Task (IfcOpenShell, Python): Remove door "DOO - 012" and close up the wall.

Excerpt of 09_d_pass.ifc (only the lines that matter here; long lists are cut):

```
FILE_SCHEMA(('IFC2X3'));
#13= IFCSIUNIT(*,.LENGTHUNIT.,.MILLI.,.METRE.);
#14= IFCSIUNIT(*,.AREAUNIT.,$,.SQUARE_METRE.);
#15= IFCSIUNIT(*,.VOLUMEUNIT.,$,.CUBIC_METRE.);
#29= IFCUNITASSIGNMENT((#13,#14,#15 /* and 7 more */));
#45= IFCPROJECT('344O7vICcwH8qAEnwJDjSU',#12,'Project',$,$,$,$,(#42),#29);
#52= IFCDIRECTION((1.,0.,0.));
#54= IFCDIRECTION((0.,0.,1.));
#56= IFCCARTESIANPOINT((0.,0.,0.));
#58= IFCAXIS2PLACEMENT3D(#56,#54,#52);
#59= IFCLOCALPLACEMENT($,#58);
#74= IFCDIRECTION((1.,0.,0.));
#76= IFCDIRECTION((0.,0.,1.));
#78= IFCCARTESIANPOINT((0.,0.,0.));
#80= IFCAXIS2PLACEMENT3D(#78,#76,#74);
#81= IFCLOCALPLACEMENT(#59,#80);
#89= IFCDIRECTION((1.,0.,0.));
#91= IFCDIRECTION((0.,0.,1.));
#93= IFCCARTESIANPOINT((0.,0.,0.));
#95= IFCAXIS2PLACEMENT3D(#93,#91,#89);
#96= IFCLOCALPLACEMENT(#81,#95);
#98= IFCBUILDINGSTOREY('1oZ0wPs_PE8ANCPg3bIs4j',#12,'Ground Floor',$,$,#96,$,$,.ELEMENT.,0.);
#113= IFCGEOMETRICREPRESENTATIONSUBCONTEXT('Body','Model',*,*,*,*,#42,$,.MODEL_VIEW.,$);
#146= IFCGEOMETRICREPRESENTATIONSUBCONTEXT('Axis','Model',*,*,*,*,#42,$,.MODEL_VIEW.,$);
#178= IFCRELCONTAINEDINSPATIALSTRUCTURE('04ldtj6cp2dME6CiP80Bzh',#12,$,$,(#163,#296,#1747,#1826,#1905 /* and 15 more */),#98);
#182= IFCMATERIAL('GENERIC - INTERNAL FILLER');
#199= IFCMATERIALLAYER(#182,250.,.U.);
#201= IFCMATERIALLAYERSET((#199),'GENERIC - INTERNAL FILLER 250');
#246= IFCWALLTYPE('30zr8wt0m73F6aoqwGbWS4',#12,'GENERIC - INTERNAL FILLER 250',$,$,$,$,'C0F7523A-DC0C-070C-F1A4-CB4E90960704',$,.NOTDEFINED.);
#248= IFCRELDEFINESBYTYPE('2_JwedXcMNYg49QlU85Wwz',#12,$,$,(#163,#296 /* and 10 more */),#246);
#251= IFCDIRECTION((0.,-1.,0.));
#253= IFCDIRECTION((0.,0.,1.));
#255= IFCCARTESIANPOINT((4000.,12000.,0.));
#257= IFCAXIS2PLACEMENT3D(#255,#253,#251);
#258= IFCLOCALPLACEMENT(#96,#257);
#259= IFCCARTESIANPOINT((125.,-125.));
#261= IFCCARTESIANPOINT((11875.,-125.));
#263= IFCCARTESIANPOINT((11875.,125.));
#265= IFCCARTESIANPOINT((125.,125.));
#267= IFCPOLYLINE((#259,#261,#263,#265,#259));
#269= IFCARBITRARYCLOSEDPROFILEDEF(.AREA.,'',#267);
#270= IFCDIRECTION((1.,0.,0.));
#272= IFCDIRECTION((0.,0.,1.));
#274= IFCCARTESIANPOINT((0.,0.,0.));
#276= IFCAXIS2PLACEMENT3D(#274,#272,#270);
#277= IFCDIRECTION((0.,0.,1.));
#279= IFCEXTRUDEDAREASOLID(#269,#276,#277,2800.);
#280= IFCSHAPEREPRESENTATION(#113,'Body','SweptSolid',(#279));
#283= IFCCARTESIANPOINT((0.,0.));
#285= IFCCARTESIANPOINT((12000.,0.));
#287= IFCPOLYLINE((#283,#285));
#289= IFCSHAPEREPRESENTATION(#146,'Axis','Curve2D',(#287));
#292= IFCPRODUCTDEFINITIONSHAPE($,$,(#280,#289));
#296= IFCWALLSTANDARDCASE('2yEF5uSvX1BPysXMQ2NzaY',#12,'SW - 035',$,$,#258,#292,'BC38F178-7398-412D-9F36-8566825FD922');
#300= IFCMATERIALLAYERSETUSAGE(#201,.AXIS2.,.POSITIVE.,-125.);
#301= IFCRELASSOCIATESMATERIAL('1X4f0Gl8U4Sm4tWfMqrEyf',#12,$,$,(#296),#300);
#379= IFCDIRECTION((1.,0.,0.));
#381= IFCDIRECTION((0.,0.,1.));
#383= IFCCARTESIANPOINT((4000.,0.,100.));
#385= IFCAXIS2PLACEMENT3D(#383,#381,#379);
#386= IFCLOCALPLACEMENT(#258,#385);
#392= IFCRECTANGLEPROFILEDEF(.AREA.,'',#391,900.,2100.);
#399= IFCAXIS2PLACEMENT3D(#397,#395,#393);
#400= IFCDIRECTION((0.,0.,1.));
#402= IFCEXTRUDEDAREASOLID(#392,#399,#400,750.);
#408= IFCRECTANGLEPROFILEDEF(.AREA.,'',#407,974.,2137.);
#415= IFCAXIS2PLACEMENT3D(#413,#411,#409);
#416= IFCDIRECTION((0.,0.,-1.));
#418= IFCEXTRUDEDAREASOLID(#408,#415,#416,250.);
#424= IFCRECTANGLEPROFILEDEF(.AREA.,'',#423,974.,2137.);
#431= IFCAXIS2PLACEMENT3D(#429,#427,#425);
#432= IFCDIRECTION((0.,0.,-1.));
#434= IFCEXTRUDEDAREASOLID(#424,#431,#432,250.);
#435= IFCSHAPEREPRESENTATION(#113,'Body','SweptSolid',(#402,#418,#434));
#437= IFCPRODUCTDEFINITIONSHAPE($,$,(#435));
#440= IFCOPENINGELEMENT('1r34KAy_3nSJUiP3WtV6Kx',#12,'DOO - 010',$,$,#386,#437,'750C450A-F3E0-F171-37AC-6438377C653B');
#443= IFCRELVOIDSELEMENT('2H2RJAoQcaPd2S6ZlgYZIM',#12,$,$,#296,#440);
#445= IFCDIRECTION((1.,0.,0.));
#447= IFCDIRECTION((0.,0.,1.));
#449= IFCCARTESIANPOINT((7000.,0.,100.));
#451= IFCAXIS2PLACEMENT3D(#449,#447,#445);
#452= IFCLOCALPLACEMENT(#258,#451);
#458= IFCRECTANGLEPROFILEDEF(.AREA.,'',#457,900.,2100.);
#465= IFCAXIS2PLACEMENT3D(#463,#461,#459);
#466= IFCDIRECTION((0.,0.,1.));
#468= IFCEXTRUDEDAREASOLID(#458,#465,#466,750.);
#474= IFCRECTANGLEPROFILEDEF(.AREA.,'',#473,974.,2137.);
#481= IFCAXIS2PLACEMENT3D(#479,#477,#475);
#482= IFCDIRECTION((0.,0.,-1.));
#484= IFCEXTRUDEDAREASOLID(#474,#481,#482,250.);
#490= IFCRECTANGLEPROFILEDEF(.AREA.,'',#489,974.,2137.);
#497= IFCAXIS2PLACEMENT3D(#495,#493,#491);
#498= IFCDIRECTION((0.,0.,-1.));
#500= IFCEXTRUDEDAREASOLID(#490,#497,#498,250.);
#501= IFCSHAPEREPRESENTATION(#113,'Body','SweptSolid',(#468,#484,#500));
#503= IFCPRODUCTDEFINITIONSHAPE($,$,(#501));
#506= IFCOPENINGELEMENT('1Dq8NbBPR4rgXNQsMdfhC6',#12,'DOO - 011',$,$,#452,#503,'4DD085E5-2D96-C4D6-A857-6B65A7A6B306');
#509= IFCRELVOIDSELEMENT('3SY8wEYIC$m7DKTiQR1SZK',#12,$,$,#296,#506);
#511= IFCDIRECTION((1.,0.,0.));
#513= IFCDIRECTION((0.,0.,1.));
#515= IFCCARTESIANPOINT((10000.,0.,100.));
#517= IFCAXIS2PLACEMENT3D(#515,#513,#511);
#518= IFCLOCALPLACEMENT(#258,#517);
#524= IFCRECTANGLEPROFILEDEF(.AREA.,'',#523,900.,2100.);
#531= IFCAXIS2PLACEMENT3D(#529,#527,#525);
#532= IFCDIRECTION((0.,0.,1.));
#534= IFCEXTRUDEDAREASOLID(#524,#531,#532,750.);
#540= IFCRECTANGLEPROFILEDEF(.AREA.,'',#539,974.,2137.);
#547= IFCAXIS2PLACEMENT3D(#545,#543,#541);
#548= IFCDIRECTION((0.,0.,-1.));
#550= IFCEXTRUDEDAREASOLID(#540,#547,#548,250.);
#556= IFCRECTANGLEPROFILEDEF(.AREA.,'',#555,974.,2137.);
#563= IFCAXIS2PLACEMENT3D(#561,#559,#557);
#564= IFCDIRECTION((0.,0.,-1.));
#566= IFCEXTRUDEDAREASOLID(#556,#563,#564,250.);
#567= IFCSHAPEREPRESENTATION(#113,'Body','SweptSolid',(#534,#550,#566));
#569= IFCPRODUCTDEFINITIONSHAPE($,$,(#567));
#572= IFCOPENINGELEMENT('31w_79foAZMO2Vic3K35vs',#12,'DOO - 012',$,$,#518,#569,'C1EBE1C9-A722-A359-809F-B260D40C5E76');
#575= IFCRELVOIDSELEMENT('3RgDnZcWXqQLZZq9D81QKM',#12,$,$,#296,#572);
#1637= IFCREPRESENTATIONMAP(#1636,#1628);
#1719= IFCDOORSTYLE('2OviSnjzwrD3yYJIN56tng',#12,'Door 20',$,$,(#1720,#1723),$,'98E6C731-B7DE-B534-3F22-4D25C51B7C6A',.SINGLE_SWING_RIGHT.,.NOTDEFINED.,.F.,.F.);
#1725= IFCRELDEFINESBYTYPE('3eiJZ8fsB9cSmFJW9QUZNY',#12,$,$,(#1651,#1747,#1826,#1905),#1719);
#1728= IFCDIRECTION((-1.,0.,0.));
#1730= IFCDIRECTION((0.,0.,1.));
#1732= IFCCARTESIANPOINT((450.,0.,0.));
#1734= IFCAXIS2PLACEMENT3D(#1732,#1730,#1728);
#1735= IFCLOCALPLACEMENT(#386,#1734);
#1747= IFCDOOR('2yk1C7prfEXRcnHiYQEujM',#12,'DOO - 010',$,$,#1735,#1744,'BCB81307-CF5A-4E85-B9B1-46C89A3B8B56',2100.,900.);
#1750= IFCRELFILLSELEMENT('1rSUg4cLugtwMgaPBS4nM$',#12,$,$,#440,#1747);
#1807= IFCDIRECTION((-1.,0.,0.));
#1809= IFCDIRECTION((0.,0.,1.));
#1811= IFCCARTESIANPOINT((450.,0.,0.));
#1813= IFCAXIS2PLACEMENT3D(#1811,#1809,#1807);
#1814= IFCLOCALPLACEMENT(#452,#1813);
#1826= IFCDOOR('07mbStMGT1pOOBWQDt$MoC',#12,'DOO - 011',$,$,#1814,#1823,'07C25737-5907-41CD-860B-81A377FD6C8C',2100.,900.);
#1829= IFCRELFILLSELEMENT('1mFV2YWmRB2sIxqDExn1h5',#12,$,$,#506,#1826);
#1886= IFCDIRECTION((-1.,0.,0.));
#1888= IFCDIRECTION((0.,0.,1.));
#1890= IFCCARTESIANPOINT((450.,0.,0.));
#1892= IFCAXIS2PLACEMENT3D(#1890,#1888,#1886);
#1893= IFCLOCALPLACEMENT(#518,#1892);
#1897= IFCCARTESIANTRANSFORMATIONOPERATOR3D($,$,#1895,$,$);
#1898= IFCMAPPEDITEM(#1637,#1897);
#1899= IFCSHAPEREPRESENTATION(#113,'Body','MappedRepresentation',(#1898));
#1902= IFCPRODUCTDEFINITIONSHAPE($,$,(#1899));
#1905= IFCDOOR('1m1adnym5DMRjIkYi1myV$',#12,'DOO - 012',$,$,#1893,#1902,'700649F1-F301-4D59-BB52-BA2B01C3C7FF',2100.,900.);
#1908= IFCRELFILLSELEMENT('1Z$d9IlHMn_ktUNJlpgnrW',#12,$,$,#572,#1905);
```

```python
import ifcopenshell
import ifcopenshell.api.feature
import ifcopenshell.api.root
import ifcopenshell.geom
import ifcopenshell.util.shape

model = ifcopenshell.open("09_d_pass.ifc")
settings = ifcopenshell.geom.settings()


def volume(element):
    """Net volume in cubic metres, openings subtracted."""
    shape = ifcopenshell.geom.create_shape(settings, element)
    return ifcopenshell.util.shape.get_volume(shape.geometry)


door = model.by_guid("1m1adnym5DMRjIkYi1myV$")
opening = door.FillsVoids[0].RelatingOpeningElement
wall = opening.VoidsElements[0].RelatingBuildingElement
before = volume(wall)

ifcopenshell.api.root.remove_product(model, product=door)
ifcopenshell.api.feature.remove_feature(model, feature=opening)

after = volume(wall)

print(f"wall volume {before:.3f} -> {after:.3f} m3")

model.write("09_d_pass_v2.ifc")
```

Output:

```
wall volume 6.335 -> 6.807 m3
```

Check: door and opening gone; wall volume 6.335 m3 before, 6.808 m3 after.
